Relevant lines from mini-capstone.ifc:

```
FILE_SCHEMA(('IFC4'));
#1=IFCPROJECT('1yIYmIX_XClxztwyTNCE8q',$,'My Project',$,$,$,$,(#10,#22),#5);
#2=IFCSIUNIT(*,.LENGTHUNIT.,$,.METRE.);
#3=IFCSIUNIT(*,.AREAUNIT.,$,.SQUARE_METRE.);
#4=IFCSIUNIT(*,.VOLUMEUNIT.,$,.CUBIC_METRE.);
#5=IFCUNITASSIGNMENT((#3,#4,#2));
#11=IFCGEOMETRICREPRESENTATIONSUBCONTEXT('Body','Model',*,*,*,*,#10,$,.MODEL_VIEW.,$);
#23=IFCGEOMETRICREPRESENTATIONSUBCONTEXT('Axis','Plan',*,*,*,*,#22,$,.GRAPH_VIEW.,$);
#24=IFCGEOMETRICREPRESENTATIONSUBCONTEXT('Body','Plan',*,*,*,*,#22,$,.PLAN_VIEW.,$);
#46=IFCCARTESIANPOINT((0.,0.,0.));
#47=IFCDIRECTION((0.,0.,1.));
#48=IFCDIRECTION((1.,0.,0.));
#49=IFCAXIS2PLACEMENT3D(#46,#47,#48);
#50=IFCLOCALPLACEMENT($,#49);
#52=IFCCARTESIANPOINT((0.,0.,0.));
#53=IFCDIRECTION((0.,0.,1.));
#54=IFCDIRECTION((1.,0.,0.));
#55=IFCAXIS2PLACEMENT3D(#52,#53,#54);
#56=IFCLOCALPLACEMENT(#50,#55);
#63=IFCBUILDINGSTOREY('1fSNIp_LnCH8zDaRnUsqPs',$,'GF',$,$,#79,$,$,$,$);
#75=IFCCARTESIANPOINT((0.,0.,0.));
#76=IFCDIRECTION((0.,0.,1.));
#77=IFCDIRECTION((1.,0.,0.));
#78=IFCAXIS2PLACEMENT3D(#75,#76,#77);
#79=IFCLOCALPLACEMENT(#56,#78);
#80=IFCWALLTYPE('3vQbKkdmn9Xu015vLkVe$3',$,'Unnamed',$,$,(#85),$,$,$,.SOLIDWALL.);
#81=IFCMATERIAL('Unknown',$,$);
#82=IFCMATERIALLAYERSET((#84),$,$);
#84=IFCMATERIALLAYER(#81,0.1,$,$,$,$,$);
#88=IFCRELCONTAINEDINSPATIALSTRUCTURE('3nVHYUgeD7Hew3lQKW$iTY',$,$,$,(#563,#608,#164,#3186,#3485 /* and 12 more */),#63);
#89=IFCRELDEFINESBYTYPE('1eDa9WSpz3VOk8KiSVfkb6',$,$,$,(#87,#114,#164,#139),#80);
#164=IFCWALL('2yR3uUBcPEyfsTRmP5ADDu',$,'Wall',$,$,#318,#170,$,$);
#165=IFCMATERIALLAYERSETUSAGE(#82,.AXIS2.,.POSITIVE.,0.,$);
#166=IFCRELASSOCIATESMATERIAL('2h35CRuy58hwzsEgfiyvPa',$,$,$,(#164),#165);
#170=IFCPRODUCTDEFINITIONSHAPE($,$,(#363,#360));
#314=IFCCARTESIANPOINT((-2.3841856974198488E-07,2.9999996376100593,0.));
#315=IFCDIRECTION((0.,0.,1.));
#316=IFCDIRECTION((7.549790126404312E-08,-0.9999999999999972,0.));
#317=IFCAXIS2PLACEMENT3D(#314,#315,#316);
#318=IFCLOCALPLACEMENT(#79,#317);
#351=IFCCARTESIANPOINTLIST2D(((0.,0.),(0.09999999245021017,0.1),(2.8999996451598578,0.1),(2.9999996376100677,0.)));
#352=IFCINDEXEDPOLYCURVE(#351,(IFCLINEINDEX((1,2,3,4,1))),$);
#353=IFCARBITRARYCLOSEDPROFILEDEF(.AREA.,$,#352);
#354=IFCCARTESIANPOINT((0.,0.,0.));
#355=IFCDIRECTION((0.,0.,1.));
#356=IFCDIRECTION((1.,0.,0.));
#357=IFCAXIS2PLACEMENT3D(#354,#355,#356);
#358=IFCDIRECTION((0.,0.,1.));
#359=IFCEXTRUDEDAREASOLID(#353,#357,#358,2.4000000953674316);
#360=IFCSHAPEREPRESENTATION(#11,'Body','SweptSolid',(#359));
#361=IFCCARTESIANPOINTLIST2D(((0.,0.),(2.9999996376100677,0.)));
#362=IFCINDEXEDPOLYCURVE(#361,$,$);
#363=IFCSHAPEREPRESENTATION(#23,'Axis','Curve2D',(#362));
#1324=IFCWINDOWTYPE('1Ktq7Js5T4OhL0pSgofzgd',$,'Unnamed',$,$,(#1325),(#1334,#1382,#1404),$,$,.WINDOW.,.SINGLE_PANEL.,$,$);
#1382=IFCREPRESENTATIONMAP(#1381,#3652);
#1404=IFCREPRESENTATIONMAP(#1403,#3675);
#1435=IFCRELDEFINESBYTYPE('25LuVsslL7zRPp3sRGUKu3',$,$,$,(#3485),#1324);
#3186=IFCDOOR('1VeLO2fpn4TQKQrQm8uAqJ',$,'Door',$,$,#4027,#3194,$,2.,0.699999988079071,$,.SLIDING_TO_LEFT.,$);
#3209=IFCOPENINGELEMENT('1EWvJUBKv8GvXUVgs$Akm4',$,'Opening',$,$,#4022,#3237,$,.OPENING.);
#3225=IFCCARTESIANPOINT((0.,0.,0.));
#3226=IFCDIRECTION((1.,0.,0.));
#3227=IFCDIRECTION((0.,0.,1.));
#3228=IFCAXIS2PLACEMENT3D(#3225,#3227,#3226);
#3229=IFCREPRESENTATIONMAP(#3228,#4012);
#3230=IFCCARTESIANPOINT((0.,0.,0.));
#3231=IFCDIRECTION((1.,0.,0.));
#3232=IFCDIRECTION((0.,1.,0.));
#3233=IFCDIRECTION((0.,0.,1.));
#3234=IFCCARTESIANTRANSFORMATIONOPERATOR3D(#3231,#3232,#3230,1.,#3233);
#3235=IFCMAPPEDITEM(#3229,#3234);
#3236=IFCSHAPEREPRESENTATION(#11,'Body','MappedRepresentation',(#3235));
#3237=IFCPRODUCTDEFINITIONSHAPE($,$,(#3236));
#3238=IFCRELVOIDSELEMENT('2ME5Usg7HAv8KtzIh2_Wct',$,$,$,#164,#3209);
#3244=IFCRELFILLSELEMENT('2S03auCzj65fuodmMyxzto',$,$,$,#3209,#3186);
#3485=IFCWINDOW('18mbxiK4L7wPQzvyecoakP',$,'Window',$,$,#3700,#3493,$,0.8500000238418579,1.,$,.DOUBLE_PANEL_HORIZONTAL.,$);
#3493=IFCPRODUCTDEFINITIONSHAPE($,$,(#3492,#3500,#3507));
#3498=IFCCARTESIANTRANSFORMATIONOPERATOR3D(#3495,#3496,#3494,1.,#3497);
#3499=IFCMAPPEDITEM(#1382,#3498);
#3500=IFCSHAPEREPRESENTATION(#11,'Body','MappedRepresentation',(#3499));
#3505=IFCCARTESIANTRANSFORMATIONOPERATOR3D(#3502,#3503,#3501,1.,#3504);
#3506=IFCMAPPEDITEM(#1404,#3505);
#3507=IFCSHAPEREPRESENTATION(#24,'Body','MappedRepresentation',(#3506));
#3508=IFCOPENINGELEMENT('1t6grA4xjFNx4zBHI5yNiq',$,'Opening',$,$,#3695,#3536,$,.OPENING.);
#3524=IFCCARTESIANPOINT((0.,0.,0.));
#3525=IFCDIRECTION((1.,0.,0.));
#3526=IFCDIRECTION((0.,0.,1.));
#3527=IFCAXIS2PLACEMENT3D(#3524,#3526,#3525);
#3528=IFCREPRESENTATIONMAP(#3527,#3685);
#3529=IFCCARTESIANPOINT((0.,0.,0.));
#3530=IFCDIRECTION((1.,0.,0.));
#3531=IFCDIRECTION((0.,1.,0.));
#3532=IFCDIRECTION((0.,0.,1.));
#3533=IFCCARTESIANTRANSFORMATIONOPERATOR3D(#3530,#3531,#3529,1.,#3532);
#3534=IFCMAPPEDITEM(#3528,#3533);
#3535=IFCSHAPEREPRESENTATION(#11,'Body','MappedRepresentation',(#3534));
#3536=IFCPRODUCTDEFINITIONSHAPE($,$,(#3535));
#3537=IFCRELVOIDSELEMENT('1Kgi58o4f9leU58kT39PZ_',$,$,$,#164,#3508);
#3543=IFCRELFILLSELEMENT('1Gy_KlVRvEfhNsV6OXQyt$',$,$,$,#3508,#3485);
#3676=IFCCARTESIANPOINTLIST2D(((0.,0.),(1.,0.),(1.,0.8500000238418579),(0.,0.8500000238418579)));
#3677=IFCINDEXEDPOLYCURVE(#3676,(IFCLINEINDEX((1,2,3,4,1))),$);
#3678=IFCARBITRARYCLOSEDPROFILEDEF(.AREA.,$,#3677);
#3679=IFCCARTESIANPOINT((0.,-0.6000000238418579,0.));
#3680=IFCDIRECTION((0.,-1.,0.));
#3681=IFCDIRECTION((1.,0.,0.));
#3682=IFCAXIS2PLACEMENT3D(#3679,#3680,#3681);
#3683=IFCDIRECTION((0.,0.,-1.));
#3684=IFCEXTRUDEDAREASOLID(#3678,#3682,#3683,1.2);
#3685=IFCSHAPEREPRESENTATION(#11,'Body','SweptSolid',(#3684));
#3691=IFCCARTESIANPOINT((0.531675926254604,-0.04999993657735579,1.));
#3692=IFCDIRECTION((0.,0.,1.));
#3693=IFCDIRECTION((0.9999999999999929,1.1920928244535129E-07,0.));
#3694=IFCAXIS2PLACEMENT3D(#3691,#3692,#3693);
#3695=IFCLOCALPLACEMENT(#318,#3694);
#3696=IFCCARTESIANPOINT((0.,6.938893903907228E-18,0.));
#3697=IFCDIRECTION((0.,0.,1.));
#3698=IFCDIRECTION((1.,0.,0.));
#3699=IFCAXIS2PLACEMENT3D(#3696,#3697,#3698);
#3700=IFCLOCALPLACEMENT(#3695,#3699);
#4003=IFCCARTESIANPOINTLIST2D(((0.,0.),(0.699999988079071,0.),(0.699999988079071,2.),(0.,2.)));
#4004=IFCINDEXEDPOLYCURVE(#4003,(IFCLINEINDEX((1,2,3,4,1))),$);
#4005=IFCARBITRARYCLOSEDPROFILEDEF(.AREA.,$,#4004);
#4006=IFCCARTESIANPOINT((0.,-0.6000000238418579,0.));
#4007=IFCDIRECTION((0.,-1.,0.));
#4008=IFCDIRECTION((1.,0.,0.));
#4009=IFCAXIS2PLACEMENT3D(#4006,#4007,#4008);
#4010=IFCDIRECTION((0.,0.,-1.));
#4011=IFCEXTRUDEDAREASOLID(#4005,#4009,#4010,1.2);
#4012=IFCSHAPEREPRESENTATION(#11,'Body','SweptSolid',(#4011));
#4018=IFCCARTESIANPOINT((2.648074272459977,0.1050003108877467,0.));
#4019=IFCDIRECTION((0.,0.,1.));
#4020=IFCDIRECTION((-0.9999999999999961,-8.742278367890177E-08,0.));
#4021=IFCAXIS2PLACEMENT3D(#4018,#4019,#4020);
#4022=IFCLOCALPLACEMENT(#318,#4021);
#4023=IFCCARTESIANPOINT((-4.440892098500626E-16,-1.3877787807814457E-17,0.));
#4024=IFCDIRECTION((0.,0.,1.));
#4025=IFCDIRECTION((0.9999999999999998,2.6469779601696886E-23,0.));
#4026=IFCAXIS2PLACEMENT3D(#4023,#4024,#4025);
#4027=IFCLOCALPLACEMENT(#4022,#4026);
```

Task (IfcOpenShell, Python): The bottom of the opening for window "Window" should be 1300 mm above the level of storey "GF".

```python
import numpy as np
import ifcopenshell
import ifcopenshell.api.geometry
import ifcopenshell.geom
import ifcopenshell.util.element
import ifcopenshell.util.placement
import ifcopenshell.util.shape
import ifcopenshell.util.unit

model = ifcopenshell.open("mini-capstone.ifc")
unit_scale = ifcopenshell.util.unit.calculate_unit_scale(model)

window = model.by_guid("18mbxiK4L7wPQzvyecoakP")
opening = window.FillsVoids[0].RelatingOpeningElement
storey = ifcopenshell.util.element.get_container(window, ifc_class="IfcBuildingStorey")
level = ifcopenshell.util.placement.get_local_placement(storey.ObjectPlacement)[2, 3]

# The opening's origin need not be at the sill, so measure its lowest point.
shape = ifcopenshell.geom.create_shape(ifcopenshell.geom.settings(), opening)
bottom = ifcopenshell.util.shape.get_shape_bottom_elevation(shape, shape.geometry) / unit_scale
dz = level + 1.3 - bottom

shift = np.array([0.0, 0.0, dz])
# The window is placed relative to its opening, so it follows when the opening moves.
matrix = ifcopenshell.util.placement.get_local_placement(opening.ObjectPlacement)
matrix[:3, 3] += shift
ifcopenshell.api.geometry.edit_object_placement(
    model, product=opening, matrix=matrix, is_si=False, should_transform_children=True
)

print(f"moved by {dz * unit_scale:+.3f} m")

model.write("mini-capstone_v2.ifc")
```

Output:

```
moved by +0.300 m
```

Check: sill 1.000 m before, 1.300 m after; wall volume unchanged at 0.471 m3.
